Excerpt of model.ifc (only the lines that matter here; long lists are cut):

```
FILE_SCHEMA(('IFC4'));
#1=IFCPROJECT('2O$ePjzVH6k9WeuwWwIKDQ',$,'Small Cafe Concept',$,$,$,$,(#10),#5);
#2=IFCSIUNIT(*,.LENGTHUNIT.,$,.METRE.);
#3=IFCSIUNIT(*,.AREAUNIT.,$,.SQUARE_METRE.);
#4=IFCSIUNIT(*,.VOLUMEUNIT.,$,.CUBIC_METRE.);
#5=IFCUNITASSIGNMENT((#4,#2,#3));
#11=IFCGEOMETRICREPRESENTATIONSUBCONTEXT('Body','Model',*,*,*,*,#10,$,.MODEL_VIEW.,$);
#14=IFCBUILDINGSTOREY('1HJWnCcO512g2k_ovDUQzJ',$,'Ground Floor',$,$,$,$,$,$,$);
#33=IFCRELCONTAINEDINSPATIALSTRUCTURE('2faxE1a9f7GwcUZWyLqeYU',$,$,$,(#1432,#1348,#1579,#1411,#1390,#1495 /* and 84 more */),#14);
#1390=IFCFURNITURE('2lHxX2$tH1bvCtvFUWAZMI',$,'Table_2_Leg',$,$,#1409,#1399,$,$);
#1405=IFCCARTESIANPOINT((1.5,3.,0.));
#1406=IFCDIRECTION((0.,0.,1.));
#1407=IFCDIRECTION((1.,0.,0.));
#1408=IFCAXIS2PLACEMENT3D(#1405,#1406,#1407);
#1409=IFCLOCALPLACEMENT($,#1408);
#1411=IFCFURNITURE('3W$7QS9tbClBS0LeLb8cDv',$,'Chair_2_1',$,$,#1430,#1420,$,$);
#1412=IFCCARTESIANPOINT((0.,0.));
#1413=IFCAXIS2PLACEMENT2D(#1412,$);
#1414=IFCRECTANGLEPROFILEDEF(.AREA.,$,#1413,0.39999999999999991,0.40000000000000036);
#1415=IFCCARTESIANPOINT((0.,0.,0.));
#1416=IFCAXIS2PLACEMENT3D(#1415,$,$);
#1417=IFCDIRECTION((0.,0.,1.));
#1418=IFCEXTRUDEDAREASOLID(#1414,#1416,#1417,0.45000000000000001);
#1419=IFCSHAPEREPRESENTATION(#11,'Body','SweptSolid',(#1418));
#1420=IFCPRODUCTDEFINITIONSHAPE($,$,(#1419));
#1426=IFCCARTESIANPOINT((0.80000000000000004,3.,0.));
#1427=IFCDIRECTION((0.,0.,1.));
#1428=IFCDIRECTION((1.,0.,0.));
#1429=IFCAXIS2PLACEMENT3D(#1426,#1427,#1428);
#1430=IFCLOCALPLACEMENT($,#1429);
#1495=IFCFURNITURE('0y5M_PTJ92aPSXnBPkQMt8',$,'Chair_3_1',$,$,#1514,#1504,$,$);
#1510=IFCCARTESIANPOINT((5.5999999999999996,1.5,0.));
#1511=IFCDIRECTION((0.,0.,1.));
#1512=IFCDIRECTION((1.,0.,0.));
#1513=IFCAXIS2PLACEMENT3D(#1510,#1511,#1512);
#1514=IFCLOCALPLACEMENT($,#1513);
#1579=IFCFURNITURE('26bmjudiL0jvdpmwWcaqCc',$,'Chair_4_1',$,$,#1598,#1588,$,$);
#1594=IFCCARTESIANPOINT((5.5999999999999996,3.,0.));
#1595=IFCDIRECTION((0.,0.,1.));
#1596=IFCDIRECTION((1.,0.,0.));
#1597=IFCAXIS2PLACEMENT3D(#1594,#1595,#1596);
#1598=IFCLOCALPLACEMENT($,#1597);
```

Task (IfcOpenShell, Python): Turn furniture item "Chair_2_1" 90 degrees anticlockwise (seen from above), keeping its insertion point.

```python
import ifcopenshell
import ifcopenshell.api.geometry
import ifcopenshell.util.placement

model = ifcopenshell.open("model.ifc")

item = model.by_id(1411)
matrix = ifcopenshell.util.placement.get_local_placement(item.ObjectPlacement)
matrix = matrix @ ifcopenshell.util.placement.rotation(90, "Z")
ifcopenshell.api.geometry.edit_object_placement(model, product=item, matrix=matrix, is_si=False)

print(ifcopenshell.util.placement.get_local_placement(item.ObjectPlacement).round(3) + 0.0)

model.write("model_rev.ifc")
```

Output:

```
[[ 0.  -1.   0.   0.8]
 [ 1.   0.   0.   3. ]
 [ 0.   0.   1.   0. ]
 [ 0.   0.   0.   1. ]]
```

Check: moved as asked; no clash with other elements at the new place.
